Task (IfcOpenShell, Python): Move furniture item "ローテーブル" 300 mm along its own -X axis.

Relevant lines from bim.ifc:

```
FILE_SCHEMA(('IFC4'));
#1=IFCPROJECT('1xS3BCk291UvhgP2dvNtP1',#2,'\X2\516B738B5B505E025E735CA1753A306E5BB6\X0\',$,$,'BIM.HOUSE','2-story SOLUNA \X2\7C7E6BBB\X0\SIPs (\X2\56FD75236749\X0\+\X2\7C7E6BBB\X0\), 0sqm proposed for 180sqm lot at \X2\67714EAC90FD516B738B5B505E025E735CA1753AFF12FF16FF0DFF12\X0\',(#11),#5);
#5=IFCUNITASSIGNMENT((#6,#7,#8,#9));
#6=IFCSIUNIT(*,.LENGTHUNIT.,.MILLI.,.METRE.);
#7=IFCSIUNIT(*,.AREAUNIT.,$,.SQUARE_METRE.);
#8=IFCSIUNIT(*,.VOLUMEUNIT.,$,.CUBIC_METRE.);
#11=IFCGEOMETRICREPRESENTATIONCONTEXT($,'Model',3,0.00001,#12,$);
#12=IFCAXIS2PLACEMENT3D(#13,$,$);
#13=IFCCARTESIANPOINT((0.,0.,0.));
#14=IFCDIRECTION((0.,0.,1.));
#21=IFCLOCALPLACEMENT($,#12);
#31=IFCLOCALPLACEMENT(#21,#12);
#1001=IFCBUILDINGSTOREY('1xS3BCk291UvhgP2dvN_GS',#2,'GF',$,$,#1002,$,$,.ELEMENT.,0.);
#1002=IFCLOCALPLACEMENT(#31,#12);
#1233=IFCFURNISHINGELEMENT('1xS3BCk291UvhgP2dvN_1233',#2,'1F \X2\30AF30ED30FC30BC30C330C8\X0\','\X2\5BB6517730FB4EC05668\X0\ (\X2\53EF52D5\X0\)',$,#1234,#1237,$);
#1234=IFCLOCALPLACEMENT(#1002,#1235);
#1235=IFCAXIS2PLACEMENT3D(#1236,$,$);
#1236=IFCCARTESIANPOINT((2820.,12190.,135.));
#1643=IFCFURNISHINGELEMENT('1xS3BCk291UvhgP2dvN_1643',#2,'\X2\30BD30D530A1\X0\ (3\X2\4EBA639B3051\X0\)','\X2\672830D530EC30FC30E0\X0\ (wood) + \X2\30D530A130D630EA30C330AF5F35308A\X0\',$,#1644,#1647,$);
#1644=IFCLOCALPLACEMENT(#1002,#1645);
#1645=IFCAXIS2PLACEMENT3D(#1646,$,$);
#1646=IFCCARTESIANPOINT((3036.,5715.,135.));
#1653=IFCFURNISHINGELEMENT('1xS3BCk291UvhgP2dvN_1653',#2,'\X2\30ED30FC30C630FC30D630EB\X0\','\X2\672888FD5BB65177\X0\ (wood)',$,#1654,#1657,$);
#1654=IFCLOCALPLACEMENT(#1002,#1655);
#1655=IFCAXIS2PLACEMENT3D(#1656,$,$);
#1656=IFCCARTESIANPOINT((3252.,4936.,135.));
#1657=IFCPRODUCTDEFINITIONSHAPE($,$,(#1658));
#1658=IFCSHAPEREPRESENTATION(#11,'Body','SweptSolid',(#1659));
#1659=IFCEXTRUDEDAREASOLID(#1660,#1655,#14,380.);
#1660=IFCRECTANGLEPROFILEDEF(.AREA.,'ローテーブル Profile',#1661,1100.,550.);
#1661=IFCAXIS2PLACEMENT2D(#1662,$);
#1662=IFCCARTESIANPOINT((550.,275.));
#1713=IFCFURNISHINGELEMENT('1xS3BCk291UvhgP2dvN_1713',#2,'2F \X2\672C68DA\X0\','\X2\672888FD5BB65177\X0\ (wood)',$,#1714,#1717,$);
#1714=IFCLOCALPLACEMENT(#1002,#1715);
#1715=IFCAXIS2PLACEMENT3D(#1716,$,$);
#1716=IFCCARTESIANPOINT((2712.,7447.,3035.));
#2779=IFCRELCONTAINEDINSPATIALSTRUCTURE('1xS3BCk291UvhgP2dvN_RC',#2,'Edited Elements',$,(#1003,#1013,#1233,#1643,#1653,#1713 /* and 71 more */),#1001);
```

```python
import ifcopenshell
import ifcopenshell.api.geometry
import ifcopenshell.util.placement

model = ifcopenshell.open("bim.ifc")

item = model.by_guid("1xS3BCk291UvhgP2dvN_1653")
matrix = ifcopenshell.util.placement.get_local_placement(item.ObjectPlacement)
matrix[:3, 3] -= matrix[:3, 0] * 300.0
ifcopenshell.api.geometry.edit_object_placement(model, product=item, matrix=matrix, is_si=False)

print(ifcopenshell.util.placement.get_local_placement(item.ObjectPlacement).round(3) + 0.0)

model.write("bim-out.ifc")
```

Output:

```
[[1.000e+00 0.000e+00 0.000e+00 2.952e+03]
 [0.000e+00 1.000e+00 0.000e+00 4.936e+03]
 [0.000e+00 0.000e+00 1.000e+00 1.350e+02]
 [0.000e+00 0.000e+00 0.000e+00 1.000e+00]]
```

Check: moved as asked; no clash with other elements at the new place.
